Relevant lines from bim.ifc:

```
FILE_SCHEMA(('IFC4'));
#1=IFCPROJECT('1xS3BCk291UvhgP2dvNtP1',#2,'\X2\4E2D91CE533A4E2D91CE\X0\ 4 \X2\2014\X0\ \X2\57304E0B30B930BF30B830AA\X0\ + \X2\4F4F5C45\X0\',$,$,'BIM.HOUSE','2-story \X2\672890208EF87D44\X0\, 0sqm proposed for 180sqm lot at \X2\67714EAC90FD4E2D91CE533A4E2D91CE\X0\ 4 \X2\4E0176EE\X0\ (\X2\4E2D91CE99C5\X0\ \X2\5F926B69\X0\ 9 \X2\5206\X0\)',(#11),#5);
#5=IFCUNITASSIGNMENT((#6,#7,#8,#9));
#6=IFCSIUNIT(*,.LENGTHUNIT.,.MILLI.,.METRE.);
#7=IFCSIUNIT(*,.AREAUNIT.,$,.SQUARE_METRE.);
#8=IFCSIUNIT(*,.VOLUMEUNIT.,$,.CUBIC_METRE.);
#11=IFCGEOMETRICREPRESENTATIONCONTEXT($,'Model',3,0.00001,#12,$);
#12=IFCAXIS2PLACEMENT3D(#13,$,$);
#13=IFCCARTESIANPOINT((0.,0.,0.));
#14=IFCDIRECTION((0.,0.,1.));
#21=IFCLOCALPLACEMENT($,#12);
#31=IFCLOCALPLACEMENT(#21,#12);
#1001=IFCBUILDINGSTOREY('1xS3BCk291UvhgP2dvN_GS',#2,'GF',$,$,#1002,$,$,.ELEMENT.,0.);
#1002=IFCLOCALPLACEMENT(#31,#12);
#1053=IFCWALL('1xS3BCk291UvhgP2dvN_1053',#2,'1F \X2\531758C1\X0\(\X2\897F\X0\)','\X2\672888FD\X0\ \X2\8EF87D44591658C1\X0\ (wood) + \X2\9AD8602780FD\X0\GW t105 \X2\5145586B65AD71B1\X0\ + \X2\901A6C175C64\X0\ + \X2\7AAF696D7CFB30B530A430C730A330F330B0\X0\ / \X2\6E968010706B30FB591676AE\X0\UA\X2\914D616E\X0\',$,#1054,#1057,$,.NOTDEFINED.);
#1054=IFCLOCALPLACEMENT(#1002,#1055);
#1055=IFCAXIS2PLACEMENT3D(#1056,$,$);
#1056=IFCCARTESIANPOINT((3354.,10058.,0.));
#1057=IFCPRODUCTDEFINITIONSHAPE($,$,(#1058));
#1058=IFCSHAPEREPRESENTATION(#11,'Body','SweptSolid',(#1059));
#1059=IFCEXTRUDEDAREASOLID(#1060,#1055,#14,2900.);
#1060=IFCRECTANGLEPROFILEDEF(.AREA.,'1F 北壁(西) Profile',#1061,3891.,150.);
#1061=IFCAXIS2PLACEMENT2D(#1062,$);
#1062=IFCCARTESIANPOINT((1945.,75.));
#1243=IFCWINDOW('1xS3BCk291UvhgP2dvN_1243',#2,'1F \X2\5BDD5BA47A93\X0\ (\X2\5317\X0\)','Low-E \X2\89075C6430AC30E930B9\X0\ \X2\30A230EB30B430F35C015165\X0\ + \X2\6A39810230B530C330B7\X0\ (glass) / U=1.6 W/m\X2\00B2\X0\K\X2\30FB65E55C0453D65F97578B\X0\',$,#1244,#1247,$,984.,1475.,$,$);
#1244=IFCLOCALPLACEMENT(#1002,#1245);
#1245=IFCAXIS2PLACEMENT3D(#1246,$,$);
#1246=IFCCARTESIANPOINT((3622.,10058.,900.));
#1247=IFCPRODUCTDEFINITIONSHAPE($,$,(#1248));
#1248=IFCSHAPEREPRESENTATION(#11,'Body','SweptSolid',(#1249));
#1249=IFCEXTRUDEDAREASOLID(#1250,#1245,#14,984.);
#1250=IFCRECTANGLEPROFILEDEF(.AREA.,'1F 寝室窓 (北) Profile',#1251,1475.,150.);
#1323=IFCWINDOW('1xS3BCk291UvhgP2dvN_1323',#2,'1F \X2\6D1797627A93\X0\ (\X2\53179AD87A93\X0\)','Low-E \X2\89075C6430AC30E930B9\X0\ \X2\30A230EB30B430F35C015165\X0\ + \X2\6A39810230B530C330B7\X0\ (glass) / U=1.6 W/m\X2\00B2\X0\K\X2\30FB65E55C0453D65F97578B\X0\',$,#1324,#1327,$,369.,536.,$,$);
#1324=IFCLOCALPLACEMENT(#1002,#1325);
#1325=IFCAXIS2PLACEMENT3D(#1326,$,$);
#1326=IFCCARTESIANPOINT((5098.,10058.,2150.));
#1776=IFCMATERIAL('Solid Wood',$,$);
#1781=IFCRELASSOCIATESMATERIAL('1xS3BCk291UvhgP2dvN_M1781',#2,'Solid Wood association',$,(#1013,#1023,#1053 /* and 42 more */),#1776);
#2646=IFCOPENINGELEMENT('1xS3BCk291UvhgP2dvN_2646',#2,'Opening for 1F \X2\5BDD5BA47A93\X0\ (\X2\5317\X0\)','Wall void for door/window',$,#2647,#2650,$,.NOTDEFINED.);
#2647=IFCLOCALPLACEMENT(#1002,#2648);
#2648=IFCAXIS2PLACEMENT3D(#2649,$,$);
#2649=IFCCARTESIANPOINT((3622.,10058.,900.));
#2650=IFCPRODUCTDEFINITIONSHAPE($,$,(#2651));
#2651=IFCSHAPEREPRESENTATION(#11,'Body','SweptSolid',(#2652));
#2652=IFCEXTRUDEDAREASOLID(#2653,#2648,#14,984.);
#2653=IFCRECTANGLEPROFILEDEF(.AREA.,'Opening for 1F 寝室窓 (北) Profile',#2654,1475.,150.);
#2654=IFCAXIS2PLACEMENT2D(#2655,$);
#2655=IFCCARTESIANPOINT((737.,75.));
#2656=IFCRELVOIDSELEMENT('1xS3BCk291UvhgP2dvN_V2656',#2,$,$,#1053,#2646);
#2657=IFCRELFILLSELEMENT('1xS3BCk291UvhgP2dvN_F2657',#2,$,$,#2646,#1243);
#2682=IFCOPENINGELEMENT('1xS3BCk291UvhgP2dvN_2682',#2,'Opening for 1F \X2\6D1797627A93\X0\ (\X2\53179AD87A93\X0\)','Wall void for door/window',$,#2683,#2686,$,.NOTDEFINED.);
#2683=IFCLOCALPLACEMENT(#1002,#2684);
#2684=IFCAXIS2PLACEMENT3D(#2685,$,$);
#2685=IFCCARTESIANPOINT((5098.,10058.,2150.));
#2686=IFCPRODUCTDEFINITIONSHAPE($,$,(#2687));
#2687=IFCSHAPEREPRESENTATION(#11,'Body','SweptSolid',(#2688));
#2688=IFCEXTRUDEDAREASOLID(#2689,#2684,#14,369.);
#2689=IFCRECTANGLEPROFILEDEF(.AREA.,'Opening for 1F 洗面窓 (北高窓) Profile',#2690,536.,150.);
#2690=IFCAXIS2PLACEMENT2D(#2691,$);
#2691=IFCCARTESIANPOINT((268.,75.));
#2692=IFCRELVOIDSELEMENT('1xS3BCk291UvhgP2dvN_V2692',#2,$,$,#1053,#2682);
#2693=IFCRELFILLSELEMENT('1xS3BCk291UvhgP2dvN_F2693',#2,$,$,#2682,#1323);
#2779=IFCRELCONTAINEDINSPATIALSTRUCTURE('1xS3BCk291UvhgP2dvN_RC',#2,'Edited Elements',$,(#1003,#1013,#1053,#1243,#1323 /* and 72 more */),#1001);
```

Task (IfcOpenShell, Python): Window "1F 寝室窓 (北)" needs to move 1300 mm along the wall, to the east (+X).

```python
import ifcopenshell
import ifcopenshell.api.geometry
import ifcopenshell.util.placement
import ifcopenshell.util.unit

model = ifcopenshell.open("bim.ifc")
unit_scale = ifcopenshell.util.unit.calculate_unit_scale(model)

window = model.by_guid("1xS3BCk291UvhgP2dvN_1243")
opening = window.FillsVoids[0].RelatingOpeningElement
wall = opening.VoidsElements[0].RelatingBuildingElement

wall_matrix = ifcopenshell.util.placement.get_local_placement(wall.ObjectPlacement)
shift = wall_matrix[:3, 0] * 1.3 / unit_scale
before = ifcopenshell.util.placement.get_local_placement(window.ObjectPlacement)[:3, 3].copy()

# The window is not placed relative to its opening, so move both.
for product in (opening, window):
    matrix = ifcopenshell.util.placement.get_local_placement(product.ObjectPlacement)
    matrix[:3, 3] += shift
    ifcopenshell.api.geometry.edit_object_placement(model, product=product, matrix=matrix, is_si=False)

after = ifcopenshell.util.placement.get_local_placement(window.ObjectPlacement)[:3, 3]
print("window moved by", (after - before).round(3) + 0.0)

model.write("bim-out.ifc")
```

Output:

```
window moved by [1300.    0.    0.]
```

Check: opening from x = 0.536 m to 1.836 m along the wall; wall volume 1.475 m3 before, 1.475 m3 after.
